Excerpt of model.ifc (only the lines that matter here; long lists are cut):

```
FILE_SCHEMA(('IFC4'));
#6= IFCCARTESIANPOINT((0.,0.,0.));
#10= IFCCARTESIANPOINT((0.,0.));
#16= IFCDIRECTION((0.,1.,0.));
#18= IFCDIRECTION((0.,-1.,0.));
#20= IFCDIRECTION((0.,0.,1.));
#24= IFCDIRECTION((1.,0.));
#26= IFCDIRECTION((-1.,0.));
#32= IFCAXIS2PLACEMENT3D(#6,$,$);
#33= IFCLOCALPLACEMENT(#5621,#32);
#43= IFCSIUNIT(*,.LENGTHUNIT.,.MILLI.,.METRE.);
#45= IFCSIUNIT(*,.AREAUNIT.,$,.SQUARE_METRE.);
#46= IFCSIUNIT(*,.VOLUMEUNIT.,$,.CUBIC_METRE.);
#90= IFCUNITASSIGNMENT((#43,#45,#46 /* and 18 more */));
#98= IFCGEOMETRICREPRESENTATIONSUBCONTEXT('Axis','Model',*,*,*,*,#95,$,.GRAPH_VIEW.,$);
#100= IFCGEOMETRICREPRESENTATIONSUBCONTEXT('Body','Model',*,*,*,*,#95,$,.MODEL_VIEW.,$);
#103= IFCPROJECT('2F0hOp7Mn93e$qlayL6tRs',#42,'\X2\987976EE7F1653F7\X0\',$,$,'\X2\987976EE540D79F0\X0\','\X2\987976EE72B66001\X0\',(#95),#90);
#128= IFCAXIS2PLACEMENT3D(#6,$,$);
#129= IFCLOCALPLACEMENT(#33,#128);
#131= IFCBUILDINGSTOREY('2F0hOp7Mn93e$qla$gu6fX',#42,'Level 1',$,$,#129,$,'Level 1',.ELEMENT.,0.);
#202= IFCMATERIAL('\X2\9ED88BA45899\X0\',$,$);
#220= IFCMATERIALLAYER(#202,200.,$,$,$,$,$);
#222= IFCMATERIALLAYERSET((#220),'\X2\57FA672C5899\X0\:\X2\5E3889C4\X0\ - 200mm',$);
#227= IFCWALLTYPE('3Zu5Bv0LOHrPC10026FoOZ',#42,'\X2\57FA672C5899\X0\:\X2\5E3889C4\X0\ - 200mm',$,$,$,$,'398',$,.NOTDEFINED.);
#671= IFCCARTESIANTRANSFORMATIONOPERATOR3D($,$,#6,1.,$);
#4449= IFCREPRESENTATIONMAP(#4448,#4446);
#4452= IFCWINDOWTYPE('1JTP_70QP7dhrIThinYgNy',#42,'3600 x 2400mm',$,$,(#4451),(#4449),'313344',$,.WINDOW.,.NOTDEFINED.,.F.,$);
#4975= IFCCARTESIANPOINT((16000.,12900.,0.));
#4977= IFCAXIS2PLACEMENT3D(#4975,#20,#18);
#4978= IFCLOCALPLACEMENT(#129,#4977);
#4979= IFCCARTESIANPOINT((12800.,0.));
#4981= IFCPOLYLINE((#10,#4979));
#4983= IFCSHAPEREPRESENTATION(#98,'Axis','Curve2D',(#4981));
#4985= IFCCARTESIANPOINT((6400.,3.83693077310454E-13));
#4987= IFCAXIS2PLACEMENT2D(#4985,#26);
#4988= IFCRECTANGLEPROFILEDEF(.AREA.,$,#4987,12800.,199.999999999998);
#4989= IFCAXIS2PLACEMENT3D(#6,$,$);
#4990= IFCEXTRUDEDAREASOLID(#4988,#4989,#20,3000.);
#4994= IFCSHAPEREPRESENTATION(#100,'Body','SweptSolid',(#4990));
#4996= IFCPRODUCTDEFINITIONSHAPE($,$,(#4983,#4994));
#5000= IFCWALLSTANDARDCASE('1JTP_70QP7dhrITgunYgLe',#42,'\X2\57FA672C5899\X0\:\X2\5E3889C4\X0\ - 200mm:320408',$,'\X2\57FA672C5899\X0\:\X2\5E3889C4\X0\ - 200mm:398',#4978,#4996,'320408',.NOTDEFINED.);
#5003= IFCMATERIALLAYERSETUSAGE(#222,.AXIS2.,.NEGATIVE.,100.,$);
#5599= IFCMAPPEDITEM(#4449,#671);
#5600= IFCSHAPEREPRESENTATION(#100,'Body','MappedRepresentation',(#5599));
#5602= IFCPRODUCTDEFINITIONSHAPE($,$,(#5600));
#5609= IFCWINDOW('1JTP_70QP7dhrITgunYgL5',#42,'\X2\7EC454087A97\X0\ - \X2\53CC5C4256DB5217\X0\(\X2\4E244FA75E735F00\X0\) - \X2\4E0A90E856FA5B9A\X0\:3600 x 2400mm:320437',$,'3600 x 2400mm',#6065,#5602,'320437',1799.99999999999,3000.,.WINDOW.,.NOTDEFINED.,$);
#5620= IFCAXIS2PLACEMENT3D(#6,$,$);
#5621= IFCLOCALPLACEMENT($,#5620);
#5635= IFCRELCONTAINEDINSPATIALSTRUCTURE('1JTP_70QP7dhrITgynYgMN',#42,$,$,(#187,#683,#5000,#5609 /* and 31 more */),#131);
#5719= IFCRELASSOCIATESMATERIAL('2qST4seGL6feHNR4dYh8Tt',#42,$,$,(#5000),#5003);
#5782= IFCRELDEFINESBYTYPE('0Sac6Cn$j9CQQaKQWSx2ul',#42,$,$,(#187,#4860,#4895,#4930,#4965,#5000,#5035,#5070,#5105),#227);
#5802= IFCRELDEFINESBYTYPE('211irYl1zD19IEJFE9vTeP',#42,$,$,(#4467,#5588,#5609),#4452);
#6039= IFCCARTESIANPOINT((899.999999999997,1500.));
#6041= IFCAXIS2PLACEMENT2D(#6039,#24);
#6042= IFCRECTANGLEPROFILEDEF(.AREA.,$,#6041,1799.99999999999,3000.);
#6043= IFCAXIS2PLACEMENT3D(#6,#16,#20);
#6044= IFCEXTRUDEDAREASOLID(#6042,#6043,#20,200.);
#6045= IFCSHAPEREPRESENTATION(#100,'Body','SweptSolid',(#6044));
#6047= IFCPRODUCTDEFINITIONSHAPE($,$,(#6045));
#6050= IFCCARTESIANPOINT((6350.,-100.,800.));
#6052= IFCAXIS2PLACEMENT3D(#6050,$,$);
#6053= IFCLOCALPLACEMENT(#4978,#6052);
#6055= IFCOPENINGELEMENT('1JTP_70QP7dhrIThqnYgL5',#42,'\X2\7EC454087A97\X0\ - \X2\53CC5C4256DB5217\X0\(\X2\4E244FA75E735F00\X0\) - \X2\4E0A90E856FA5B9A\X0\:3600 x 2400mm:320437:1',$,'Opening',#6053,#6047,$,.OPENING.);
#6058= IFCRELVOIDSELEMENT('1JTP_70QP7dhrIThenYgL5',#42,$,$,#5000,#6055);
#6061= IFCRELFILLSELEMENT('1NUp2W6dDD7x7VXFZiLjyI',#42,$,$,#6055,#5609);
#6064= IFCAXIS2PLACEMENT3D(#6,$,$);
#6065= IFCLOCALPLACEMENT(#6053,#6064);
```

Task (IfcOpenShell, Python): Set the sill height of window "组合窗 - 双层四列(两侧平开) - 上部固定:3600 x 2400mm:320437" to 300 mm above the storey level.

```python
import numpy as np
import ifcopenshell
import ifcopenshell.api.geometry
import ifcopenshell.geom
import ifcopenshell.util.element
import ifcopenshell.util.placement
import ifcopenshell.util.shape
import ifcopenshell.util.unit

model = ifcopenshell.open("model.ifc")
unit_scale = ifcopenshell.util.unit.calculate_unit_scale(model)

window = model.by_guid("1JTP_70QP7dhrITgunYgL5")
opening = window.FillsVoids[0].RelatingOpeningElement
storey = ifcopenshell.util.element.get_container(window, ifc_class="IfcBuildingStorey")
level = ifcopenshell.util.placement.get_local_placement(storey.ObjectPlacement)[2, 3]

# The opening's origin need not be at the sill, so measure its lowest point.
shape = ifcopenshell.geom.create_shape(ifcopenshell.geom.settings(), opening)
bottom = ifcopenshell.util.shape.get_shape_bottom_elevation(shape, shape.geometry) / unit_scale
dz = level + 0.3 / unit_scale - bottom

shift = np.array([0.0, 0.0, dz])
# The window is placed relative to its opening, so it follows when the opening moves.
matrix = ifcopenshell.util.placement.get_local_placement(opening.ObjectPlacement)
matrix[:3, 3] += shift
ifcopenshell.api.geometry.edit_object_placement(
    model, product=opening, matrix=matrix, is_si=False, should_transform_children=True
)

print(f"moved by {dz * unit_scale:+.3f} m")

model.write("model_edited.ifc")
```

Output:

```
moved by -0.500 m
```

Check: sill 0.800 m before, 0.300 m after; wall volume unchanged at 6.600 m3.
